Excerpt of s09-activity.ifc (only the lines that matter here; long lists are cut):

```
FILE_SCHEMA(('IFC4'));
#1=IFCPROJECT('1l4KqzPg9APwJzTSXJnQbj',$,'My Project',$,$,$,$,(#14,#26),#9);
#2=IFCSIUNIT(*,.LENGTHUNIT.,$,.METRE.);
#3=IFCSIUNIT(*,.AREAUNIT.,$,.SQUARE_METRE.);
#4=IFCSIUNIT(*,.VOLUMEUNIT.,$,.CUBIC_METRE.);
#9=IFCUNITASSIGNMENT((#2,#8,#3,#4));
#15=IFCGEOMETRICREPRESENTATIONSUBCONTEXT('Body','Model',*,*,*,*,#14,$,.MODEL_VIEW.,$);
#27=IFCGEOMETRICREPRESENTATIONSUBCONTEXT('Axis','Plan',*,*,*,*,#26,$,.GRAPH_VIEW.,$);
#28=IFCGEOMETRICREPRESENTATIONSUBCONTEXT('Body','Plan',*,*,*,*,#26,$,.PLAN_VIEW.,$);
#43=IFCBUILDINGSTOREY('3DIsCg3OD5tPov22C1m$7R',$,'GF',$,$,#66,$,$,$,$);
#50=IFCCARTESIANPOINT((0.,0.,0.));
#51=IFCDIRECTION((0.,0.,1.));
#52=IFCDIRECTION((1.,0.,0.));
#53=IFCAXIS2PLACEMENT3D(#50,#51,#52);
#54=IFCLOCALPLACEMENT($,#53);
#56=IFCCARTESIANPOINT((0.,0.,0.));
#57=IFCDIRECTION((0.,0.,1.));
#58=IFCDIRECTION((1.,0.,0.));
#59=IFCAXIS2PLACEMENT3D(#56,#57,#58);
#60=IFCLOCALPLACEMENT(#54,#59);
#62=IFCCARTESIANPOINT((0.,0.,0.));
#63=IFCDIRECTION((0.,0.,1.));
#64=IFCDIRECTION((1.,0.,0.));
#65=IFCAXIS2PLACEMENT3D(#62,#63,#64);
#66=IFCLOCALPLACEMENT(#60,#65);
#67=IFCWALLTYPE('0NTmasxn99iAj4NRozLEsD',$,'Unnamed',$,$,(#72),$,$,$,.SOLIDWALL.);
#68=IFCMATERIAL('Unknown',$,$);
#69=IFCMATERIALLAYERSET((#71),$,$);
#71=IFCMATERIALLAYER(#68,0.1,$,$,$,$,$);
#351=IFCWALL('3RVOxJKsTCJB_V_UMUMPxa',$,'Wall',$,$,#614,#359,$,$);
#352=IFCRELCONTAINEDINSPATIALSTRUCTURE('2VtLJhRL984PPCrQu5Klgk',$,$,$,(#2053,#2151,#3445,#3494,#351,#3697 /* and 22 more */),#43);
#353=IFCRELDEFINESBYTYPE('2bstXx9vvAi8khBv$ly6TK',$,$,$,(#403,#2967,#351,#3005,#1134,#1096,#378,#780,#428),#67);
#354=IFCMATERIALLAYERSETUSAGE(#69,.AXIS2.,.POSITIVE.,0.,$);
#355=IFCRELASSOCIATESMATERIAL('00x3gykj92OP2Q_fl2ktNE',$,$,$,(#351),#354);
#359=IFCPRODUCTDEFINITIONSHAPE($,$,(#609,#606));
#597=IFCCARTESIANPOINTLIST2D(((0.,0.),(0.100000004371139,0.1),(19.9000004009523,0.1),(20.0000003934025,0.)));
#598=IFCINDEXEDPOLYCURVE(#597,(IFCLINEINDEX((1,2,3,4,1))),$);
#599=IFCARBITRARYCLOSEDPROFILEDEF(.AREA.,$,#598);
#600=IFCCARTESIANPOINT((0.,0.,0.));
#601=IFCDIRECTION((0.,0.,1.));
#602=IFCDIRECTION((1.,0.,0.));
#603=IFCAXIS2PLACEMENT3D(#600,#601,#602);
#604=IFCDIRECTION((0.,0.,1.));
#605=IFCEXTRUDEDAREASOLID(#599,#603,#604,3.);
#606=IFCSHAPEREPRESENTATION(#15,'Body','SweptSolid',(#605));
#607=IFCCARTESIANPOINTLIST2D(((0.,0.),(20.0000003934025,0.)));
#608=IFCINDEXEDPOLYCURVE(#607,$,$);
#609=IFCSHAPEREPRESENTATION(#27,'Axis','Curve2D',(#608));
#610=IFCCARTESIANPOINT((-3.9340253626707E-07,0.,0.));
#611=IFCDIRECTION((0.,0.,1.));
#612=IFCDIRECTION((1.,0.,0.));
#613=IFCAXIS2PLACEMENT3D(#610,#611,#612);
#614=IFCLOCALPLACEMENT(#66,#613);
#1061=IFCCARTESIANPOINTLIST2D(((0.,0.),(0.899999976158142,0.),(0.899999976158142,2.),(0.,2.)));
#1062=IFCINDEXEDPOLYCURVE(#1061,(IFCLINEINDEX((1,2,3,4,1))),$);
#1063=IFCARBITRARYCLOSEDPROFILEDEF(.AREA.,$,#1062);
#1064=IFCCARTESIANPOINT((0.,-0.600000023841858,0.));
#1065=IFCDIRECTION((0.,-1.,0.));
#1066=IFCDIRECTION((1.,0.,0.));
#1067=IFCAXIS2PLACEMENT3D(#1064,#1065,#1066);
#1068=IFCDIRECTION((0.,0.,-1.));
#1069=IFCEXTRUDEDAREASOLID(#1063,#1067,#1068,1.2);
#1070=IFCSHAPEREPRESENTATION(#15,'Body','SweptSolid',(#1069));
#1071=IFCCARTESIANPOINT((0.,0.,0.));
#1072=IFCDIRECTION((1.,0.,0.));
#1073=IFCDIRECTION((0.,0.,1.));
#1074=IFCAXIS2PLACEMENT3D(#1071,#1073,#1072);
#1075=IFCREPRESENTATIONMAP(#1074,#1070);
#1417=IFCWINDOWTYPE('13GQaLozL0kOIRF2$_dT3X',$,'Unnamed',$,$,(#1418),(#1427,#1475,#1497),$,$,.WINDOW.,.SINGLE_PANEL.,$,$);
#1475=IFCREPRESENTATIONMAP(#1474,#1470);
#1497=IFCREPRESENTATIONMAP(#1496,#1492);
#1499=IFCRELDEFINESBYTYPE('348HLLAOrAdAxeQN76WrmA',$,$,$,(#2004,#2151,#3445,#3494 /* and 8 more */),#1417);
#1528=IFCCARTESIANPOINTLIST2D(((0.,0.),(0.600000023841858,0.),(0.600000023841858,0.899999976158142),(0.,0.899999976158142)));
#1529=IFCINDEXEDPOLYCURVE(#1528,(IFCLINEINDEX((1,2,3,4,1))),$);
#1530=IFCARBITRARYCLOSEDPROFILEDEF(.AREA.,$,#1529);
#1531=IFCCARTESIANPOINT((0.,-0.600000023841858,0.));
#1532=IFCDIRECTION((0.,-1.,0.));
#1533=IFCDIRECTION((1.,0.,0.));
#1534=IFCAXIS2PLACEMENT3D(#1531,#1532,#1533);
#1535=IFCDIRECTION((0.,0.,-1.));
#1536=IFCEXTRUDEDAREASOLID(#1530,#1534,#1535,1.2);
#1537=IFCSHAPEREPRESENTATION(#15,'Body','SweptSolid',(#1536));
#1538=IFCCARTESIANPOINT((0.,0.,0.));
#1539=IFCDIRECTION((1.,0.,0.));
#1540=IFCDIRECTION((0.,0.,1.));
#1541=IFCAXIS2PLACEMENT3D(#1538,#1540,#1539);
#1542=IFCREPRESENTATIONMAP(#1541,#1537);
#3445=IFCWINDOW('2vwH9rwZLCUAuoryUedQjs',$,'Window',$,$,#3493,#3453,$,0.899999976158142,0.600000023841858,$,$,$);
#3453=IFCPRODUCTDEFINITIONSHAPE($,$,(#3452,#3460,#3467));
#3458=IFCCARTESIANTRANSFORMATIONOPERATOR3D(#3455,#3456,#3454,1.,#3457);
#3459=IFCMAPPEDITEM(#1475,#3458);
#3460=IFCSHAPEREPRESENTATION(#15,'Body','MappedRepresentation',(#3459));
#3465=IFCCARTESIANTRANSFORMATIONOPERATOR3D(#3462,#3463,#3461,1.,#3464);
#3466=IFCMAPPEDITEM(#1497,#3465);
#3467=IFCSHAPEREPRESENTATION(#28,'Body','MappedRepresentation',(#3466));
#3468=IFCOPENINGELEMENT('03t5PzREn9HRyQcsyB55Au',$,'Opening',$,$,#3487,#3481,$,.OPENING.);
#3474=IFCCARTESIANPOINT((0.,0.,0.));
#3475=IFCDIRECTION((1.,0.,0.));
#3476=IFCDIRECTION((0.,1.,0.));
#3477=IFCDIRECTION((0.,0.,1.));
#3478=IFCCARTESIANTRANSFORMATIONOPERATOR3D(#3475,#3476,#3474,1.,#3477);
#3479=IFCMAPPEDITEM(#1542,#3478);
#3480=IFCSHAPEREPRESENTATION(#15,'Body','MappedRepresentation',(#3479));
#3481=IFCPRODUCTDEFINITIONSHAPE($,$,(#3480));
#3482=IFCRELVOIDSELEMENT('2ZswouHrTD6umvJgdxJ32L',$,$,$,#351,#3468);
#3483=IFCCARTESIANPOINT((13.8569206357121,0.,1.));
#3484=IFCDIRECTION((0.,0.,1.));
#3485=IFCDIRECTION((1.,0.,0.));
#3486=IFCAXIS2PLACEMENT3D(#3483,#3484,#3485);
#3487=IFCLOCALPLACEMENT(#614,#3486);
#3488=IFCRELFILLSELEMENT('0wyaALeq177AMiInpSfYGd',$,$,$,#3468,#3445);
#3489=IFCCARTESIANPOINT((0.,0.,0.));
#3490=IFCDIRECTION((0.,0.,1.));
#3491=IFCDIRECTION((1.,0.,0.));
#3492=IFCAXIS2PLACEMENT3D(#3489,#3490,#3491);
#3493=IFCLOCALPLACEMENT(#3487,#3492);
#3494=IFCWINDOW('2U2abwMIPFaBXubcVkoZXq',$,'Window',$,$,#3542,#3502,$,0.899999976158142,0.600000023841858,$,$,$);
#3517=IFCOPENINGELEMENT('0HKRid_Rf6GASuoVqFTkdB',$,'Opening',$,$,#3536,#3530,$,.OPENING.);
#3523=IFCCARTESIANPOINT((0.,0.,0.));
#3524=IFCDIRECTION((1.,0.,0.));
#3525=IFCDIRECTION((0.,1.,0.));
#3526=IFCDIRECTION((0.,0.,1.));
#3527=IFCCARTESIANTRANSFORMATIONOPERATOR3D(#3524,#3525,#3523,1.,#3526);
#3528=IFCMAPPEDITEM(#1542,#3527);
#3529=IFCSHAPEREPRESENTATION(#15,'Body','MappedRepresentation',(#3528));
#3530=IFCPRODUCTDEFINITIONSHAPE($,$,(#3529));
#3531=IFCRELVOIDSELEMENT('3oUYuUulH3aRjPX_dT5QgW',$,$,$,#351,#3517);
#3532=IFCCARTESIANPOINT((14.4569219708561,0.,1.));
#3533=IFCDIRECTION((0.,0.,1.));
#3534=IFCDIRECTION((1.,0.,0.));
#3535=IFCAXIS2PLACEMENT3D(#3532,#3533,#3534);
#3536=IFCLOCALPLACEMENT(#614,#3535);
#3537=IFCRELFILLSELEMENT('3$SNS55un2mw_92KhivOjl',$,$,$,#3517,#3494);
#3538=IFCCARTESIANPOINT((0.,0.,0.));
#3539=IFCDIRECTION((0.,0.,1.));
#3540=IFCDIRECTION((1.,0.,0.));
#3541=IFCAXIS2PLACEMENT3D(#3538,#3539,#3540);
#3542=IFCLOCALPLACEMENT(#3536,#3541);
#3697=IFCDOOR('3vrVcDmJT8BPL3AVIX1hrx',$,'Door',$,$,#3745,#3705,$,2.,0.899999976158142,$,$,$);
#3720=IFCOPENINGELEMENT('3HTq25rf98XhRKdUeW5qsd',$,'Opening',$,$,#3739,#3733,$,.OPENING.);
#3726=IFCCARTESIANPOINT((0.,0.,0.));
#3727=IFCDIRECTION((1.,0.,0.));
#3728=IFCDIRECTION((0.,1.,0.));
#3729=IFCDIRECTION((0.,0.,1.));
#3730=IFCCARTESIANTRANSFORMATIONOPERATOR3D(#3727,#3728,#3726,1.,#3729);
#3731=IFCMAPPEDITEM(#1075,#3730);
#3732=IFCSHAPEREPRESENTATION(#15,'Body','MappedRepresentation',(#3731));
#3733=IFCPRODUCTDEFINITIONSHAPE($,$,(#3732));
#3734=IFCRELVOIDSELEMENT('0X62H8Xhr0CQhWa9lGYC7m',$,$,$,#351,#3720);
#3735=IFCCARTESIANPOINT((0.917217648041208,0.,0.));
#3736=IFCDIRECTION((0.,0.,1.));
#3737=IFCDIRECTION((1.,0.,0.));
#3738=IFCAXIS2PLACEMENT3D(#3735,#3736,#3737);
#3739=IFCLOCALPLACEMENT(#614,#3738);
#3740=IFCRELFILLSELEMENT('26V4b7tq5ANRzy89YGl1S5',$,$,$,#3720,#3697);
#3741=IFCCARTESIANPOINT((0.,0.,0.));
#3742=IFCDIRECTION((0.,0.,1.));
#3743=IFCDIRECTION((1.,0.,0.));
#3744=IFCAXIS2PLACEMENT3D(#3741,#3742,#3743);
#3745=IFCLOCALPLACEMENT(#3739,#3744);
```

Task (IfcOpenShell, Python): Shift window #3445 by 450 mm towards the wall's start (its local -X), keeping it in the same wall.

```python
import ifcopenshell
import ifcopenshell.api.geometry
import ifcopenshell.util.placement

model = ifcopenshell.open("s09-activity.ifc")

window = model.by_guid("2vwH9rwZLCUAuoryUedQjs")
opening = window.FillsVoids[0].RelatingOpeningElement
wall = opening.VoidsElements[0].RelatingBuildingElement

wall_matrix = ifcopenshell.util.placement.get_local_placement(wall.ObjectPlacement)
shift = wall_matrix[:3, 0] * -0.45
before = ifcopenshell.util.placement.get_local_placement(window.ObjectPlacement)[:3, 3].copy()

# The window is placed relative to its opening, so it follows when the opening moves.
matrix = ifcopenshell.util.placement.get_local_placement(opening.ObjectPlacement)
matrix[:3, 3] += shift
ifcopenshell.api.geometry.edit_object_placement(
    model, product=opening, matrix=matrix, is_si=False, should_transform_children=True
)

after = ifcopenshell.util.placement.get_local_placement(window.ObjectPlacement)[:3, 3]
print("window moved by", (after - before).round(3) + 0.0)

model.write("s09-activity-out.ifc")
```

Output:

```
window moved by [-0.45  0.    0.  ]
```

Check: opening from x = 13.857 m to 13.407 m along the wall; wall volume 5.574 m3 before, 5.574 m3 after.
